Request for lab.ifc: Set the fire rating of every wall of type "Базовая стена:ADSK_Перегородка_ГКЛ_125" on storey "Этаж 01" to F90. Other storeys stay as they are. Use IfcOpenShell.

First a look at what the model holds.

```python
import ifcopenshell
import ifcopenshell.util.element

model = ifcopenshell.open("lab.ifc")
print(model.schema)
storey = next(s for s in model.by_type("IfcBuildingStorey") if s.Name == "Этаж 01")
walls = [e for e in ifcopenshell.util.element.get_decomposition(storey) if e.is_a("IfcWall")]
seen = {}
for e in walls:
    element_type = ifcopenshell.util.element.get_type(e)
    key = (element_type.Name if element_type != e and element_type else None, ifcopenshell.util.element.get_pset(e, "Pset_WallCommon", "FireRating"))
    seen[key] = seen.get(key, 0) + 1
for (name, value), count in sorted(seen.items(), key=str):
    print(count, "x", name, "|", value)
```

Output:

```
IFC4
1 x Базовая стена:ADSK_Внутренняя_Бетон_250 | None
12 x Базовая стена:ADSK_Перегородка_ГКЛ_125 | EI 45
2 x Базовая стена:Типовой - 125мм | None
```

```python
import ifcopenshell
import ifcopenshell.api.pset
import ifcopenshell.util.element

model = ifcopenshell.open("lab.ifc")

storey = next(s for s in model.by_type("IfcBuildingStorey") if s.Name == "Этаж 01")
walls = [e for e in ifcopenshell.util.element.get_decomposition(storey) if e.is_a("IfcWall")]

count = 0
for e in walls:
    element_type = ifcopenshell.util.element.get_type(e)
    if element_type in (None, e) or element_type.Name != "Базовая стена:ADSK_Перегородка_ГКЛ_125":
        continue
    # add_pset returns the element's existing set when there is one.
    pset = ifcopenshell.api.pset.add_pset(model, product=e, name="Pset_WallCommon")
    ifcopenshell.api.pset.edit_pset(model, pset=pset, properties={"FireRating": "F90"})
    count += 1

print(count, "walls updated")

model.write("lab_rev.ifc")
```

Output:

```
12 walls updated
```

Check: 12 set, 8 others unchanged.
